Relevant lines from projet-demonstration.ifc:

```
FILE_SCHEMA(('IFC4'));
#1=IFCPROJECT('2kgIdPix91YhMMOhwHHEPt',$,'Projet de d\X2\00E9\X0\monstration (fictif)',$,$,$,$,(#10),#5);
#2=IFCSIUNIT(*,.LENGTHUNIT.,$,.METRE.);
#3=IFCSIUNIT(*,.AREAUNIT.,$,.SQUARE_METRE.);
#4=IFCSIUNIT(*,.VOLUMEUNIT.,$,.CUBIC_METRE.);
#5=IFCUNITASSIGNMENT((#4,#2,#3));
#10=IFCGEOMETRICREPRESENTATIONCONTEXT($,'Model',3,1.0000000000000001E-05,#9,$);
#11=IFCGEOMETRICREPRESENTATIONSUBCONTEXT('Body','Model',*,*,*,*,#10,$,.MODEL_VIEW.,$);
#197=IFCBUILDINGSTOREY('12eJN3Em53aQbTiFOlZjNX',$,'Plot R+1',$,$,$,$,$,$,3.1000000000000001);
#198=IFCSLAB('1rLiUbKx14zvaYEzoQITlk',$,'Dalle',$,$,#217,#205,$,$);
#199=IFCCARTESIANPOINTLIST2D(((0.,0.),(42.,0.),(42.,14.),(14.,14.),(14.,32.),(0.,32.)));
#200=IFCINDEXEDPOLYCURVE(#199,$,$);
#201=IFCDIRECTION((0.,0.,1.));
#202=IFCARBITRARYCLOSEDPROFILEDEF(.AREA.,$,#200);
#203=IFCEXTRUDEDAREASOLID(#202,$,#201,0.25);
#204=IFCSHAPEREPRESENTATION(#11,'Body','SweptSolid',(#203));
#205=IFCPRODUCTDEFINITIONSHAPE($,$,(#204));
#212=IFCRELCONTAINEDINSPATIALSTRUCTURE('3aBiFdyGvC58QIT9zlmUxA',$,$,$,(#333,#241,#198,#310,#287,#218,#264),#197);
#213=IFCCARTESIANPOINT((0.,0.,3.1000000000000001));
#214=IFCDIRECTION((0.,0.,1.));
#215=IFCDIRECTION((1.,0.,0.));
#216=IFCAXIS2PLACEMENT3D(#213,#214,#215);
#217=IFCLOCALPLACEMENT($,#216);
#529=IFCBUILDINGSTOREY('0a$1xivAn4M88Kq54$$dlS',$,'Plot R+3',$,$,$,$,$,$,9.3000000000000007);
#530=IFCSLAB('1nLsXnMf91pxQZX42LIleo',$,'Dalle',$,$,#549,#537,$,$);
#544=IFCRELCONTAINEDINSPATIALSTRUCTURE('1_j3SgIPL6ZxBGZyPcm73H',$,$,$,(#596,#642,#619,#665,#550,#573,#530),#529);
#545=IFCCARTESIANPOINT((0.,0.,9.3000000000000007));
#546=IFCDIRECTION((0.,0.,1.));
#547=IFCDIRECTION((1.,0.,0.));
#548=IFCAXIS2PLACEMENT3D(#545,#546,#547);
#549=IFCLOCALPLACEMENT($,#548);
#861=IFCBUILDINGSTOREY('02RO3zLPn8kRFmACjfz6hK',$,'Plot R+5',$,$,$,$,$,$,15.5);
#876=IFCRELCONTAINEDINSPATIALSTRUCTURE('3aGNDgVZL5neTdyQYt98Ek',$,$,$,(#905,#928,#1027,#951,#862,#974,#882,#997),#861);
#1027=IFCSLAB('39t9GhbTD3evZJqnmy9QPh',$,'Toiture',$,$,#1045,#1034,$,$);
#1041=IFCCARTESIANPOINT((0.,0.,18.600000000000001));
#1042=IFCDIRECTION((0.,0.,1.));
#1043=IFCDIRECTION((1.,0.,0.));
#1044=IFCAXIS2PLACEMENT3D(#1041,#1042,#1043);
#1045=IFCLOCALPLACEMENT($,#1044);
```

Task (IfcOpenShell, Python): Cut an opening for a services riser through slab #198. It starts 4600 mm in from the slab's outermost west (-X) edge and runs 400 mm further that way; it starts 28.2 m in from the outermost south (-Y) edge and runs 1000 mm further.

```python
import numpy as np
import ifcopenshell
import ifcopenshell.api.feature
import ifcopenshell.api.geometry
import ifcopenshell.api.root
import ifcopenshell.geom
import ifcopenshell.util.placement
import ifcopenshell.util.representation
import ifcopenshell.util.shape
import ifcopenshell.util.unit

model = ifcopenshell.open("projet-demonstration.ifc")
unit_scale = ifcopenshell.util.unit.calculate_unit_scale(model)
settings = ifcopenshell.geom.settings()


def volume(element):
    """Net volume in cubic metres, openings subtracted."""
    shape = ifcopenshell.geom.create_shape(settings, element)
    return ifcopenshell.util.shape.get_volume(shape.geometry)


slab = model.by_id(198)
before = volume(slab)

# Extent in the slab's own axes, in metres. The edges named are its -X and -Y sides.
slab_shape = ifcopenshell.geom.create_shape(settings, slab)
vertices = ifcopenshell.util.shape.get_vertices(slab_shape.geometry)
x_min, y_min, bottom = vertices.min(axis=0)
top = vertices[:, 2].max()

opening = ifcopenshell.api.root.create_entity(model, ifc_class="IfcOpeningElement", name="Services riser opening", predefined_type="OPENING")
context = ifcopenshell.util.representation.get_context(model, "Model", "Body", "MODEL_VIEW")
width, depth = 0.4, 1
outline = [(0.0, 0.0), (width, 0.0), (width, depth), (0.0, depth), (0.0, 0.0)]
# Overshoot both faces by 50 mm so the cut is clean.
shape = ifcopenshell.api.geometry.add_slab_representation(
    model, context=context, depth=top - bottom + 0.1, polyline=outline
)
ifcopenshell.api.geometry.assign_representation(model, product=opening, representation=shape)

matrix = ifcopenshell.util.placement.get_local_placement(slab.ObjectPlacement)
matrix[:, 3] = matrix @ np.append(np.array([x_min + 4.6, y_min + 28.2, bottom - 0.05]) / unit_scale, 1.0)
ifcopenshell.api.geometry.edit_object_placement(model, product=opening, matrix=matrix, is_si=False)
ifcopenshell.api.feature.add_feature(model, feature=opening, element=slab)

after = volume(slab)

print(f"slab volume {before:.3f} -> {after:.3f} m3")

model.write("projet-demonstration_rev.ifc")
```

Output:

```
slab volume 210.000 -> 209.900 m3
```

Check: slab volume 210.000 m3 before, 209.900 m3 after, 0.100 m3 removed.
